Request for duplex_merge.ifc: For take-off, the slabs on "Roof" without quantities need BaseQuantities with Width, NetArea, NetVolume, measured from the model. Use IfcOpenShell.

First a look at what the model holds.

```python
import ifcopenshell
import ifcopenshell.util.element
import ifcopenshell.util.unit

model = ifcopenshell.open("duplex_merge.ifc")
print(model.schema)
for unit_type in ("LENGTHUNIT", "AREAUNIT", "VOLUMEUNIT"):
    print(unit_type, ifcopenshell.util.unit.calculate_unit_scale(model, unit_type))
storey = next(s for s in model.by_type("IfcBuildingStorey") if s.Name == "Roof")
slabs = [e for e in ifcopenshell.util.element.get_decomposition(storey) if e.is_a("IfcSlab")]
for e in sorted(slabs, key=lambda e: e.id()):
    print(e.id(), e.is_a(), e.Name, list(ifcopenshell.util.element.get_psets(e, qtos_only=True)), sep=" | ")
```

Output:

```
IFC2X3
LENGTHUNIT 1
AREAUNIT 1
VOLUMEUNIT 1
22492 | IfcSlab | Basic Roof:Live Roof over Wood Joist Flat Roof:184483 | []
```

```python
import ifcopenshell
import ifcopenshell.api.pset
import ifcopenshell.geom
import ifcopenshell.util.element
import ifcopenshell.util.shape
import ifcopenshell.util.unit

model = ifcopenshell.open("duplex_merge.ifc")
unit_scale = ifcopenshell.util.unit.calculate_unit_scale(model)
area_scale = ifcopenshell.util.unit.calculate_unit_scale(model, "AREAUNIT")
volume_scale = ifcopenshell.util.unit.calculate_unit_scale(model, "VOLUMEUNIT")
settings = ifcopenshell.geom.settings()

storey = next(s for s in model.by_type("IfcBuildingStorey") if s.Name == "Roof")
slabs = [e for e in ifcopenshell.util.element.get_decomposition(storey) if e.is_a("IfcSlab")]

for e in sorted(slabs, key=lambda e: e.id()):
    if ifcopenshell.util.element.get_psets(e, qtos_only=True, should_inherit=False):
        continue
    # Geometry comes back in metres, in the element's own axes.
    shape = ifcopenshell.geom.create_shape(settings, e)
    values = {
        "Width": ifcopenshell.util.shape.get_z(shape.geometry) / unit_scale,
        "NetArea": ifcopenshell.util.shape.get_footprint_area(shape.geometry) / area_scale,
        "NetVolume": ifcopenshell.util.shape.get_volume(shape.geometry) / volume_scale,
    }
    qto = ifcopenshell.api.pset.add_qto(model, product=e, name="BaseQuantities")
    ifcopenshell.api.pset.edit_qto(model, qto=qto, properties=values)
    print(e.id(), {k: round(v, 3) for k, v in values.items()})

model.write("duplex_merge_v2.ifc")
```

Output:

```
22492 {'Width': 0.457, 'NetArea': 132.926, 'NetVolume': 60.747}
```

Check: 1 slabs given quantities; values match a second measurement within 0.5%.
